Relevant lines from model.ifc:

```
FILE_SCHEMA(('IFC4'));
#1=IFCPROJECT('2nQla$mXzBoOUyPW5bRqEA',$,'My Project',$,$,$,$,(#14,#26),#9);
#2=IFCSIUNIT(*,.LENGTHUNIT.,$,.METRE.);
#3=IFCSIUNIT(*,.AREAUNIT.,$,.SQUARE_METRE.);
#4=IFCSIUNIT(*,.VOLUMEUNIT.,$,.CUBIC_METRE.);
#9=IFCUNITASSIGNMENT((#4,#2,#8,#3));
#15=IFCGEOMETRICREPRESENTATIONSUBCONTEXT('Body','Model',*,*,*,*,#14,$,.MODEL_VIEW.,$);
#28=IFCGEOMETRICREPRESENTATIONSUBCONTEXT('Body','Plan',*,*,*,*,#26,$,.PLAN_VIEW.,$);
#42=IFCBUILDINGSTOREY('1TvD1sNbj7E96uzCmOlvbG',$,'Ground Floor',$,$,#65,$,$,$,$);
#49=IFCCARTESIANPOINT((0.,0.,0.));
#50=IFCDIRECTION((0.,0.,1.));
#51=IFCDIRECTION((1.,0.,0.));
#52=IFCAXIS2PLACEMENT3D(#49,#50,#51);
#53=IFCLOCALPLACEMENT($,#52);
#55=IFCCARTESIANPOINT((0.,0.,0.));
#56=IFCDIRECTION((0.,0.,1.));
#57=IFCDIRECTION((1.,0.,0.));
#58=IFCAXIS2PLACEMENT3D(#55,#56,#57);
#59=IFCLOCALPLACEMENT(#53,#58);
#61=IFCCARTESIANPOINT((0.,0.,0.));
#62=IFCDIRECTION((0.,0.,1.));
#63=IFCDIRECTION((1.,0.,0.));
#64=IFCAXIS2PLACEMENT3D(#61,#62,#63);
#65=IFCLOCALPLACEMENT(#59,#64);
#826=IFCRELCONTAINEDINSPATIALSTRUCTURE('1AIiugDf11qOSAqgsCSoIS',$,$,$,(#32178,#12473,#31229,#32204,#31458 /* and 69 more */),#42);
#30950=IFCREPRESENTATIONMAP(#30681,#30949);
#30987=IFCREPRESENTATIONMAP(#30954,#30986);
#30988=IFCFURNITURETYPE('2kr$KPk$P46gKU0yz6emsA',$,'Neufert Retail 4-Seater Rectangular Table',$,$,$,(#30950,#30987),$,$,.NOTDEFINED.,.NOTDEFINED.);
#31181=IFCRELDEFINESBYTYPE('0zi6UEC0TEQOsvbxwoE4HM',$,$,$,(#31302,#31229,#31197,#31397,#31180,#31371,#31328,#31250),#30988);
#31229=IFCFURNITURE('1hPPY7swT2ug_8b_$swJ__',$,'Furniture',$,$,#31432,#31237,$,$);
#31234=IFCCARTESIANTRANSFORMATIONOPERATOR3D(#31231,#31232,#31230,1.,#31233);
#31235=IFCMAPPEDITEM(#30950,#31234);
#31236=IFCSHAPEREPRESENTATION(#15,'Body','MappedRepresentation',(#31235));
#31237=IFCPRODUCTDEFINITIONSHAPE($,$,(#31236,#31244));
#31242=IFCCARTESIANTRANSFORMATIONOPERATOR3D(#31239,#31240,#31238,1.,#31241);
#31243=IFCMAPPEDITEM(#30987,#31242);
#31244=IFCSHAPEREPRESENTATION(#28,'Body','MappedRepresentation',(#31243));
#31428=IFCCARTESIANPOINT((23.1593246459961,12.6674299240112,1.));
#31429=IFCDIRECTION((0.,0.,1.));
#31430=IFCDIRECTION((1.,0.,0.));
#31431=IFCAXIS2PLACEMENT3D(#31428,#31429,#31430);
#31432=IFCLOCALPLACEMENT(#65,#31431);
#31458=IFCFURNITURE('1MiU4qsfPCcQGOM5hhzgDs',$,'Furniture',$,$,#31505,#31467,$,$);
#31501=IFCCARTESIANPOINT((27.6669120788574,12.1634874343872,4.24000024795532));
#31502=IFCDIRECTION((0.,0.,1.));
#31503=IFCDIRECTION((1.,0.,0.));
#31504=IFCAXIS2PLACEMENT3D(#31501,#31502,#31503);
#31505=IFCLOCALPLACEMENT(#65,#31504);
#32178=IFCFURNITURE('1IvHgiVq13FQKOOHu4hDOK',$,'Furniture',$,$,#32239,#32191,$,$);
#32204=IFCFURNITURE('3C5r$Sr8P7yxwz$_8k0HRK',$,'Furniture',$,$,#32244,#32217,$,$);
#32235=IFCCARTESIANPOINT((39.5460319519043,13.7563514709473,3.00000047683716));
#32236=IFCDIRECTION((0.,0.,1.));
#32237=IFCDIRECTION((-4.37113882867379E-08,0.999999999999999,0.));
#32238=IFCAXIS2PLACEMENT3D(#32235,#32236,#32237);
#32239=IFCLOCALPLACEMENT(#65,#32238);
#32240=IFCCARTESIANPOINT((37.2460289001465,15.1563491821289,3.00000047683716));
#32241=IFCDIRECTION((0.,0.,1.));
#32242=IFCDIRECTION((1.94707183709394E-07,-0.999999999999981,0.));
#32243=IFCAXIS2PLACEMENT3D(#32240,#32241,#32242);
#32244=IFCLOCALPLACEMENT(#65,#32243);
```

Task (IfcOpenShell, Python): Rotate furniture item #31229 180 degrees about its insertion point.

```python
import ifcopenshell
import ifcopenshell.api.geometry
import ifcopenshell.util.placement

model = ifcopenshell.open("model.ifc")

item = model.by_guid("1hPPY7swT2ug_8b_$swJ__")
matrix = ifcopenshell.util.placement.get_local_placement(item.ObjectPlacement)
matrix = matrix @ ifcopenshell.util.placement.rotation(180, "Z")
ifcopenshell.api.geometry.edit_object_placement(model, product=item, matrix=matrix, is_si=False)

print(ifcopenshell.util.placement.get_local_placement(item.ObjectPlacement).round(3) + 0.0)

model.write("model_v2.ifc")
```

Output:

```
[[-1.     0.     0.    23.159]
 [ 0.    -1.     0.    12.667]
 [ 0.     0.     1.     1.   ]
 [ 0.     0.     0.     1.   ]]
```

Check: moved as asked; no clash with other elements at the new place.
